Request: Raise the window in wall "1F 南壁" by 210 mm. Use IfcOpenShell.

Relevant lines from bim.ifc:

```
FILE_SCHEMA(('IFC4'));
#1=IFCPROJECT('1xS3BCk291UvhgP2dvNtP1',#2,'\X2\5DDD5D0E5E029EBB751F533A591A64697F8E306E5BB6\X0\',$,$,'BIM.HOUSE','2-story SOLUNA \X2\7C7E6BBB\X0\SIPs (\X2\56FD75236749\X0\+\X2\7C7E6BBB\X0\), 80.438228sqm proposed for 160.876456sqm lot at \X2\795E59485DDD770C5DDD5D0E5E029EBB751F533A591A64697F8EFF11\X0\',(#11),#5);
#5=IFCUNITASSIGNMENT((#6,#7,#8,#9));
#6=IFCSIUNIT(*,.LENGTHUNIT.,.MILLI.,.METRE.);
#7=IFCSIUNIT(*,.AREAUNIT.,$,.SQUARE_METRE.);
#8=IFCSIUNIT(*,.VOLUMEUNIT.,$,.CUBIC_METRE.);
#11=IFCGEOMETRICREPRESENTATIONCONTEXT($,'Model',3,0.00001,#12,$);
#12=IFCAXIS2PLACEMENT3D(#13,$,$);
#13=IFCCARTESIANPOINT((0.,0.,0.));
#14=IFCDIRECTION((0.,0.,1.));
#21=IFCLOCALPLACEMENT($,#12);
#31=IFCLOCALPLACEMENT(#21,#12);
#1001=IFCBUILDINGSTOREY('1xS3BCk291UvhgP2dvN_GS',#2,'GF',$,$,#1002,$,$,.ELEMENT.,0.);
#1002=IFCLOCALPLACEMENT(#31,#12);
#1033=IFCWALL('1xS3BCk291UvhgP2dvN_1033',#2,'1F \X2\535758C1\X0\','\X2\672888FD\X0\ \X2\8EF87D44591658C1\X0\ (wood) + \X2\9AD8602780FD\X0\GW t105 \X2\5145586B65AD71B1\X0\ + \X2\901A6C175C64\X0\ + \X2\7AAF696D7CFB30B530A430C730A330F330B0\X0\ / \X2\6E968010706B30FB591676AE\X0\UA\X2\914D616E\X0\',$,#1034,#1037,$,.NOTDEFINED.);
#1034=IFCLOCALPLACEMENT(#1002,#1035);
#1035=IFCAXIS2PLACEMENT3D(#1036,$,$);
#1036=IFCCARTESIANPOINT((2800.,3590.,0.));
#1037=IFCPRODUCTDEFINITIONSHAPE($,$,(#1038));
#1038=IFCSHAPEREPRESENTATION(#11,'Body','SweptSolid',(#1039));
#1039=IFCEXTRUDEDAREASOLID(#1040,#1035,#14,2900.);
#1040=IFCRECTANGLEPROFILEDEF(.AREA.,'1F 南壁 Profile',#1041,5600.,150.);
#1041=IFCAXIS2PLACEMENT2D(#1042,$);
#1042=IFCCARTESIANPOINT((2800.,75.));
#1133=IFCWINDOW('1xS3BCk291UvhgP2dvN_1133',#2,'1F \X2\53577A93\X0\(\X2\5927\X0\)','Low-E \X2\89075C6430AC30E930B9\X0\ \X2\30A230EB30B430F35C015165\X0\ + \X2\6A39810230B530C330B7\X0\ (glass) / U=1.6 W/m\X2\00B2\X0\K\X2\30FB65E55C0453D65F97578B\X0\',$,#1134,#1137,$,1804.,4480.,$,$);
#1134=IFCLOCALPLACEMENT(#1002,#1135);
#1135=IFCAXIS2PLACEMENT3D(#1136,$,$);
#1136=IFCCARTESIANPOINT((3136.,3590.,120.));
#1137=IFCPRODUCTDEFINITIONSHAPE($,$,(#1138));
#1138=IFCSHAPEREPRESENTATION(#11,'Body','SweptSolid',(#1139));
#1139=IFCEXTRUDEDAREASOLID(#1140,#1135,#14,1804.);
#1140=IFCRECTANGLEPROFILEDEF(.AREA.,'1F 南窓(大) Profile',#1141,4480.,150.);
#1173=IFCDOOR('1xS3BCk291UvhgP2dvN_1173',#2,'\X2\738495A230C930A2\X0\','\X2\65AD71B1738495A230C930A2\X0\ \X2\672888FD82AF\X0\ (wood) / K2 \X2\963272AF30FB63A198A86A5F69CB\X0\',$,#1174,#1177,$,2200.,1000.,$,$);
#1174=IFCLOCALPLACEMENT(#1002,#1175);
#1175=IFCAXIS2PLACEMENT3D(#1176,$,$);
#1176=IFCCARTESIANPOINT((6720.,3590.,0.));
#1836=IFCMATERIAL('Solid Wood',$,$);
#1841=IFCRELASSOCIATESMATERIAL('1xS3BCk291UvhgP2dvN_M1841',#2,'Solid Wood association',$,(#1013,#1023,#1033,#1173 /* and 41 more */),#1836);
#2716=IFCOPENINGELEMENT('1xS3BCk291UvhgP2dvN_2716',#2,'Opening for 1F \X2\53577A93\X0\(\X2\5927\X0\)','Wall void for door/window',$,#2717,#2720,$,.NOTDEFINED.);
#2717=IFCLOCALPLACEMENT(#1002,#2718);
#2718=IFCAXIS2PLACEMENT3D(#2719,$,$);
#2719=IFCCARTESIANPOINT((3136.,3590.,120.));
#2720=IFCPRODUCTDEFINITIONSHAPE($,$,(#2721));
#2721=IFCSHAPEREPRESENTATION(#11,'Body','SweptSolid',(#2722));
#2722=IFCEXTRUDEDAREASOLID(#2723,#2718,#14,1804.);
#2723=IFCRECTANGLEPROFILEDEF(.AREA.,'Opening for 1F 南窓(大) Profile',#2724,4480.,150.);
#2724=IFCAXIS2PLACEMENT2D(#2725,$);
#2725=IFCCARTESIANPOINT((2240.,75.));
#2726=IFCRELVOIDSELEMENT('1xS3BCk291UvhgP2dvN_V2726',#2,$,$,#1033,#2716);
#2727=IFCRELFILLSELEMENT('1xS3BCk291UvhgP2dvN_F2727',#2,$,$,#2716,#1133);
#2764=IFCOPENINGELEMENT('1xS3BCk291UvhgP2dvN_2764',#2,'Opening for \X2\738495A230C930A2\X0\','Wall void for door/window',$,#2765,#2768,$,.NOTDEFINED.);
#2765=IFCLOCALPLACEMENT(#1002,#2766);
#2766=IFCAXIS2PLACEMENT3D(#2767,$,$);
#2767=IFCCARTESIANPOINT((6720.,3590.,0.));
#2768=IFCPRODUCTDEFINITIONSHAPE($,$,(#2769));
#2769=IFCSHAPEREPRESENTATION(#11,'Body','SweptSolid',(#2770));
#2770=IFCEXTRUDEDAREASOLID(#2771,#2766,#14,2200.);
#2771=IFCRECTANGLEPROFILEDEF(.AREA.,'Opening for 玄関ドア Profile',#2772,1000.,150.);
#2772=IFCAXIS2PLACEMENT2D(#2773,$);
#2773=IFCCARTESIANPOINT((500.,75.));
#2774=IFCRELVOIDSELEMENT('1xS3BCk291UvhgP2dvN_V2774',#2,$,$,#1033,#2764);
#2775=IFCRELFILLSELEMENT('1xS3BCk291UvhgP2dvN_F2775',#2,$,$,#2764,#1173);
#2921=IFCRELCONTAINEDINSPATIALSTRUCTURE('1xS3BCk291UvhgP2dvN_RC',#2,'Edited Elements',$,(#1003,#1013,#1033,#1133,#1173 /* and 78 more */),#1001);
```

```python
import numpy as np
import ifcopenshell
import ifcopenshell.api.geometry
import ifcopenshell.util.placement
import ifcopenshell.util.unit

model = ifcopenshell.open("bim.ifc")
unit_scale = ifcopenshell.util.unit.calculate_unit_scale(model)

window = model.by_guid("1xS3BCk291UvhgP2dvN_1133")
opening = window.FillsVoids[0].RelatingOpeningElement
dz = 0.21 / unit_scale

shift = np.array([0.0, 0.0, dz])
# The window is not placed relative to its opening, so move both.
for product in (opening, window):
    matrix = ifcopenshell.util.placement.get_local_placement(product.ObjectPlacement)
    matrix[:3, 3] += shift
    ifcopenshell.api.geometry.edit_object_placement(model, product=product, matrix=matrix, is_si=False)

print(f"moved by {dz * unit_scale:+.3f} m")

model.write("bim_edited.ifc")
```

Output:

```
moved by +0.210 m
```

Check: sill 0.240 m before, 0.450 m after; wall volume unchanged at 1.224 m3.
